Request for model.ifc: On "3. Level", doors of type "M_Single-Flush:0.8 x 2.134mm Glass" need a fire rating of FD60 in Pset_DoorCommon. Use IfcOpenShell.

First a look at what the model holds.

```python
import ifcopenshell
import ifcopenshell.util.element

model = ifcopenshell.open("model.ifc")
print(model.schema)
storey = next(s for s in model.by_type("IfcBuildingStorey") if s.Name == "3. Level")
doors = [e for e in ifcopenshell.util.element.get_decomposition(storey) if e.is_a("IfcDoor")]
seen = {}
for e in doors:
    element_type = ifcopenshell.util.element.get_type(e)
    key = (element_type.Name if element_type != e and element_type else None, ifcopenshell.util.element.get_pset(e, "Pset_DoorCommon", "FireRating"))
    seen[key] = seen.get(key, 0) + 1
for (name, value), count in sorted(seen.items(), key=str):
    print(count, "x", name, "|", value)
```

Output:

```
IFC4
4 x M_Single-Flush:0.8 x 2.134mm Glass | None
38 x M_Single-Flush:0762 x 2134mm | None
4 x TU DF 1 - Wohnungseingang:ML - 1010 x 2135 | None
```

```python
import ifcopenshell
import ifcopenshell.api.pset
import ifcopenshell.util.element

model = ifcopenshell.open("model.ifc")

storey = next(s for s in model.by_type("IfcBuildingStorey") if s.Name == "3. Level")
doors = [e for e in ifcopenshell.util.element.get_decomposition(storey) if e.is_a("IfcDoor")]

count = 0
for e in doors:
    element_type = ifcopenshell.util.element.get_type(e)
    if element_type in (None, e) or element_type.Name != "M_Single-Flush:0.8 x 2.134mm Glass":
        continue
    # add_pset returns the element's existing set when there is one.
    pset = ifcopenshell.api.pset.add_pset(model, product=e, name="Pset_DoorCommon")
    ifcopenshell.api.pset.edit_pset(model, pset=pset, properties={"FireRating": "FD60"})
    count += 1

print(count, "doors updated")

model.write("model_v2.ifc")
```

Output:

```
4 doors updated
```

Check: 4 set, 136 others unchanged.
